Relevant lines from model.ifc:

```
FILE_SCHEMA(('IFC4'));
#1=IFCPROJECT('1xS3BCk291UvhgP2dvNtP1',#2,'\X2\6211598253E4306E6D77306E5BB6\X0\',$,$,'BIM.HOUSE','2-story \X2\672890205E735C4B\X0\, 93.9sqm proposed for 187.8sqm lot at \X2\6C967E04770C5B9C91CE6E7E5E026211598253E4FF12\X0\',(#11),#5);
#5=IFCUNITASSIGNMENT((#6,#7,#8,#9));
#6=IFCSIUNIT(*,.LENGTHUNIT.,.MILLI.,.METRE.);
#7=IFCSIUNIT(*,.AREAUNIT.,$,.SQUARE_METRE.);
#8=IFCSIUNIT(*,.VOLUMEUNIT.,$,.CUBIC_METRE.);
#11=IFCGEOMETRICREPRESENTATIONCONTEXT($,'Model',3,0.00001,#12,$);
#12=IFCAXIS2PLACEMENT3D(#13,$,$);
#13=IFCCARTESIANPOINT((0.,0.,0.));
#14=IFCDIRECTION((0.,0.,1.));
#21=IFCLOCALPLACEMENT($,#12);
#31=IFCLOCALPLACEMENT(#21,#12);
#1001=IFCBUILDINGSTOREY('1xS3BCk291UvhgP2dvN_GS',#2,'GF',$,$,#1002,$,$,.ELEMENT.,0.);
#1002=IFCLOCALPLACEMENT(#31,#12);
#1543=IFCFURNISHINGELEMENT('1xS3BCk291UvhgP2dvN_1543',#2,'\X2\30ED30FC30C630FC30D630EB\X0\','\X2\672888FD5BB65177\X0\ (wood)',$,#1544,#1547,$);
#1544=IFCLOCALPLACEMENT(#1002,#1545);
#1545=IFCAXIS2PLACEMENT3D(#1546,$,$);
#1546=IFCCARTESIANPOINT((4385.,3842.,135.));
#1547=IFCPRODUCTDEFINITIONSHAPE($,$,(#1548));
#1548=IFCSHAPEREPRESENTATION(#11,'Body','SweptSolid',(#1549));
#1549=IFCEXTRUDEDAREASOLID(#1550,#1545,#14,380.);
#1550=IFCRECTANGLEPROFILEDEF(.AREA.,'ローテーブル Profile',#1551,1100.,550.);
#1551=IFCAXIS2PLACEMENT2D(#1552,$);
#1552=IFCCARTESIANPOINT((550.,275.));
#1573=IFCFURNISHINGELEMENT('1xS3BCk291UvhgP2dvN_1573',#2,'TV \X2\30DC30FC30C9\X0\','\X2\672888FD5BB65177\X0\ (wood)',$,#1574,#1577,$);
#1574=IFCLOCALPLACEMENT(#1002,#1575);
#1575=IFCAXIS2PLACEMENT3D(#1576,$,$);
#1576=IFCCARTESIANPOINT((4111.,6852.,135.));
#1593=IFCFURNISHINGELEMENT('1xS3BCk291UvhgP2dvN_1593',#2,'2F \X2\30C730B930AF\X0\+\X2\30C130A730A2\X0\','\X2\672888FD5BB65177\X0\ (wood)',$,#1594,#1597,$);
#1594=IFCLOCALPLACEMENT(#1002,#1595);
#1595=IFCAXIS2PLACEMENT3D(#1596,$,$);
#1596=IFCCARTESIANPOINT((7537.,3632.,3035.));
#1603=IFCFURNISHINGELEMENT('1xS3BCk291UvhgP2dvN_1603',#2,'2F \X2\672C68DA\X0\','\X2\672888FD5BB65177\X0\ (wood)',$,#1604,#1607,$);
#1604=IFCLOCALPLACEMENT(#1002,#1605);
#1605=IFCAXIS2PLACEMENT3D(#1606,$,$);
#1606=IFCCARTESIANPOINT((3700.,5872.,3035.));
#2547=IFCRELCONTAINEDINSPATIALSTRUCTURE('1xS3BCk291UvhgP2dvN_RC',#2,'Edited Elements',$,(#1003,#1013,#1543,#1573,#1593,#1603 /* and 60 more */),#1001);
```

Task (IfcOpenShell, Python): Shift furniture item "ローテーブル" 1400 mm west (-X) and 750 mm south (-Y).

```python
import ifcopenshell
import ifcopenshell.api.geometry
import ifcopenshell.util.placement
import ifcopenshell.util.unit

model = ifcopenshell.open("model.ifc")
unit_scale = ifcopenshell.util.unit.calculate_unit_scale(model)

item = model.by_guid("1xS3BCk291UvhgP2dvN_1543")
matrix = ifcopenshell.util.placement.get_local_placement(item.ObjectPlacement)
matrix[0, 3] -= 1.4 / unit_scale
matrix[1, 3] -= 0.75 / unit_scale
ifcopenshell.api.geometry.edit_object_placement(model, product=item, matrix=matrix, is_si=False)

print(ifcopenshell.util.placement.get_local_placement(item.ObjectPlacement).round(3) + 0.0)

model.write("model_edited.ifc")
```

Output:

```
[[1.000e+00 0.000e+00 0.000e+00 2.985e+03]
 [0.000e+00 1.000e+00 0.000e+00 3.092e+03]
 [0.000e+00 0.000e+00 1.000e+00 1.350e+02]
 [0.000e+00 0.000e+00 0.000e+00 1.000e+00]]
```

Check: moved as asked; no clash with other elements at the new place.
